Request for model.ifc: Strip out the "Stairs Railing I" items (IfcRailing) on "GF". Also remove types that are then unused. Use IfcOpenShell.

First a look at what the model holds.

```python
import ifcopenshell
import ifcopenshell.util.element

model = ifcopenshell.open("model.ifc")
print(model.schema)
storey = next(s for s in model.by_type("IfcBuildingStorey") if s.Name == "GF")
railings = [e for e in ifcopenshell.util.element.get_decomposition(storey) if e.is_a("IfcRailing")]
seen = {}
for e in railings:
    element_type = ifcopenshell.util.element.get_type(e)
    name = element_type.Name if element_type not in (None, e) else None
    seen[name] = seen.get(name, 0) + 1
for name, count in sorted(seen.items(), key=str):
    print(count, "x", name)
```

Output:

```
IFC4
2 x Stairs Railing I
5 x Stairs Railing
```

```python
import ifcopenshell
import ifcopenshell.api.root
import ifcopenshell.util.element

model = ifcopenshell.open("model.ifc")

storey = next(s for s in model.by_type("IfcBuildingStorey") if s.Name == "GF")
railings = [e for e in ifcopenshell.util.element.get_decomposition(storey) if e.is_a("IfcRailing")]
targets = [e for e in railings if (t := ifcopenshell.util.element.get_type(e)) not in (None, e) and t.Name == "Stairs Railing I"]
types = {ifcopenshell.util.element.get_type(e) for e in targets} - {None, *targets}

for e in targets:
    ifcopenshell.api.root.remove_product(model, product=e)
print(len(targets), "removed")

unused = [t for t in types if not ifcopenshell.util.element.get_types(t)]
for t in unused:
    ifcopenshell.api.root.remove_product(model, product=t)
print(len(unused), "unused types removed")

model.write("model_edited.ifc")
```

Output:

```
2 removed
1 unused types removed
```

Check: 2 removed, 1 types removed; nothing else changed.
